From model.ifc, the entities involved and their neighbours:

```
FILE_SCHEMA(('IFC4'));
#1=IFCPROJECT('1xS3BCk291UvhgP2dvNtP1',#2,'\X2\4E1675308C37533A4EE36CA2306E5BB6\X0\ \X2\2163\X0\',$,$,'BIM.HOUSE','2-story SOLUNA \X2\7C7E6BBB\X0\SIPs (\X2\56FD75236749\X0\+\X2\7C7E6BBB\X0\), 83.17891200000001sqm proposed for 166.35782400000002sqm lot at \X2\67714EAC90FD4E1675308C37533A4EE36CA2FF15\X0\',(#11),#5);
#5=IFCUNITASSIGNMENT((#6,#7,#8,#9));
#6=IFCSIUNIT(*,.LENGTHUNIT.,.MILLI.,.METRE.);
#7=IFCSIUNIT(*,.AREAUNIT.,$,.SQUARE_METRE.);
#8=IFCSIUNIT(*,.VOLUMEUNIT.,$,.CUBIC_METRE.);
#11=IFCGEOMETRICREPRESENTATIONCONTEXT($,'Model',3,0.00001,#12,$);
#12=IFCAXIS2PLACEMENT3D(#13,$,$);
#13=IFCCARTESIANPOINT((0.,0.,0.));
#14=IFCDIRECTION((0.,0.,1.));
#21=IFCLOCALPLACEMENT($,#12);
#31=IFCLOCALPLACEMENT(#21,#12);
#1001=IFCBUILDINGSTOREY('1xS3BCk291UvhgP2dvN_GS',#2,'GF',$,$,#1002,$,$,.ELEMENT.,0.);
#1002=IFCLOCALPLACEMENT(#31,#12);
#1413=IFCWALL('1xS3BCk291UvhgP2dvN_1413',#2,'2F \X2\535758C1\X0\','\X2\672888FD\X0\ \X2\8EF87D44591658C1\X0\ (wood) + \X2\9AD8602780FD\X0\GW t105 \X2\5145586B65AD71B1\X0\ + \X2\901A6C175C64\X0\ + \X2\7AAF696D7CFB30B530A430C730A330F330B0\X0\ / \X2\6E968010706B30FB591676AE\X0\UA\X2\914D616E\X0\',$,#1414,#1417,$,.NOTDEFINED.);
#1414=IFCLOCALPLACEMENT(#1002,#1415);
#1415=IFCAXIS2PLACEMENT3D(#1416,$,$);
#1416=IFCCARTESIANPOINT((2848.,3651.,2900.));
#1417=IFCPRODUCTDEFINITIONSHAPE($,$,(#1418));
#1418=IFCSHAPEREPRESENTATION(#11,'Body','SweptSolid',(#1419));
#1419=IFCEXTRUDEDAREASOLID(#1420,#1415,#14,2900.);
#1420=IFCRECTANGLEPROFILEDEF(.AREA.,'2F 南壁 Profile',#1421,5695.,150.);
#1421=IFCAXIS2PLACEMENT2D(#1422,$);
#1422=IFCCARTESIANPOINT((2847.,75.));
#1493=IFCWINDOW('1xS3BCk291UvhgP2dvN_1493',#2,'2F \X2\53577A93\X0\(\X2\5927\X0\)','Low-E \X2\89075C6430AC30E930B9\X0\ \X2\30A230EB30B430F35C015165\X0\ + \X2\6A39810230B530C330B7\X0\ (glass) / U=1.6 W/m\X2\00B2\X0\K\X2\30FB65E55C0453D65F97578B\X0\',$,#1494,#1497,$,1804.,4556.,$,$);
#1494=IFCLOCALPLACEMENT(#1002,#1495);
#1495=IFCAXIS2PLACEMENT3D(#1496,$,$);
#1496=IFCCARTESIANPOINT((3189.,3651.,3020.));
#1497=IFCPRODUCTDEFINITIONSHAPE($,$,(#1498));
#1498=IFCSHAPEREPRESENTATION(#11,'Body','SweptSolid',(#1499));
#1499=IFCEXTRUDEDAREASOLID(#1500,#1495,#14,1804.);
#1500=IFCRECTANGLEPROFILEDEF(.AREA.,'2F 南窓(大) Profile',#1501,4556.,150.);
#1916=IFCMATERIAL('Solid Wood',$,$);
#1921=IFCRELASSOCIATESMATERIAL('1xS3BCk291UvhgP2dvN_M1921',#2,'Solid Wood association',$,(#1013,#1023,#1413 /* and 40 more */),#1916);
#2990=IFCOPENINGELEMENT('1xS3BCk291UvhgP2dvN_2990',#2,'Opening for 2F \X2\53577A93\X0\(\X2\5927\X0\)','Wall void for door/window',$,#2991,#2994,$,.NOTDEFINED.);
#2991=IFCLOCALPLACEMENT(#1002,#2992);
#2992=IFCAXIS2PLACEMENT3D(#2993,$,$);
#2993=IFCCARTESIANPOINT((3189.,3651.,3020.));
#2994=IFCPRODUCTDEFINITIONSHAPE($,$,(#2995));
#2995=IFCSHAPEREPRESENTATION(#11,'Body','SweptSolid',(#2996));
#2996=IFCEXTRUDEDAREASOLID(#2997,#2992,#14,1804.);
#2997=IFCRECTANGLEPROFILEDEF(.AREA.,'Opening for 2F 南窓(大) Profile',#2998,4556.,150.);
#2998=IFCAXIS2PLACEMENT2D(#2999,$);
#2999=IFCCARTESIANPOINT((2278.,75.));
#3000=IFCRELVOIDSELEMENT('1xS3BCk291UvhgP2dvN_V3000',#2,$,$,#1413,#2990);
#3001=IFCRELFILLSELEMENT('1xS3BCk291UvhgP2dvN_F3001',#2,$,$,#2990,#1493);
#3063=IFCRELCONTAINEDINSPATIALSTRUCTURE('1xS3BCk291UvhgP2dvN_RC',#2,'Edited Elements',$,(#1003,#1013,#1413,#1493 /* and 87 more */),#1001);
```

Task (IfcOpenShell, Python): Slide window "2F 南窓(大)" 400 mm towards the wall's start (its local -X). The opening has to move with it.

```python
import ifcopenshell
import ifcopenshell.api.geometry
import ifcopenshell.util.placement

model = ifcopenshell.open("model.ifc")

window = model.by_guid("1xS3BCk291UvhgP2dvN_1493")
opening = window.FillsVoids[0].RelatingOpeningElement
wall = opening.VoidsElements[0].RelatingBuildingElement

wall_matrix = ifcopenshell.util.placement.get_local_placement(wall.ObjectPlacement)
shift = wall_matrix[:3, 0] * -400.0
before = ifcopenshell.util.placement.get_local_placement(window.ObjectPlacement)[:3, 3].copy()

# The window is not placed relative to its opening, so move both.
for product in (opening, window):
    matrix = ifcopenshell.util.placement.get_local_placement(product.ObjectPlacement)
    matrix[:3, 3] += shift
    ifcopenshell.api.geometry.edit_object_placement(model, product=product, matrix=matrix, is_si=False)

after = ifcopenshell.util.placement.get_local_placement(window.ObjectPlacement)[:3, 3]
print("window moved by", (after - before).round(3) + 0.0)

model.write("model_edited.ifc")
```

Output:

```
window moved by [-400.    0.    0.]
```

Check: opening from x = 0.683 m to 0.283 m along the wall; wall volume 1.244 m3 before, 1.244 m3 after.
